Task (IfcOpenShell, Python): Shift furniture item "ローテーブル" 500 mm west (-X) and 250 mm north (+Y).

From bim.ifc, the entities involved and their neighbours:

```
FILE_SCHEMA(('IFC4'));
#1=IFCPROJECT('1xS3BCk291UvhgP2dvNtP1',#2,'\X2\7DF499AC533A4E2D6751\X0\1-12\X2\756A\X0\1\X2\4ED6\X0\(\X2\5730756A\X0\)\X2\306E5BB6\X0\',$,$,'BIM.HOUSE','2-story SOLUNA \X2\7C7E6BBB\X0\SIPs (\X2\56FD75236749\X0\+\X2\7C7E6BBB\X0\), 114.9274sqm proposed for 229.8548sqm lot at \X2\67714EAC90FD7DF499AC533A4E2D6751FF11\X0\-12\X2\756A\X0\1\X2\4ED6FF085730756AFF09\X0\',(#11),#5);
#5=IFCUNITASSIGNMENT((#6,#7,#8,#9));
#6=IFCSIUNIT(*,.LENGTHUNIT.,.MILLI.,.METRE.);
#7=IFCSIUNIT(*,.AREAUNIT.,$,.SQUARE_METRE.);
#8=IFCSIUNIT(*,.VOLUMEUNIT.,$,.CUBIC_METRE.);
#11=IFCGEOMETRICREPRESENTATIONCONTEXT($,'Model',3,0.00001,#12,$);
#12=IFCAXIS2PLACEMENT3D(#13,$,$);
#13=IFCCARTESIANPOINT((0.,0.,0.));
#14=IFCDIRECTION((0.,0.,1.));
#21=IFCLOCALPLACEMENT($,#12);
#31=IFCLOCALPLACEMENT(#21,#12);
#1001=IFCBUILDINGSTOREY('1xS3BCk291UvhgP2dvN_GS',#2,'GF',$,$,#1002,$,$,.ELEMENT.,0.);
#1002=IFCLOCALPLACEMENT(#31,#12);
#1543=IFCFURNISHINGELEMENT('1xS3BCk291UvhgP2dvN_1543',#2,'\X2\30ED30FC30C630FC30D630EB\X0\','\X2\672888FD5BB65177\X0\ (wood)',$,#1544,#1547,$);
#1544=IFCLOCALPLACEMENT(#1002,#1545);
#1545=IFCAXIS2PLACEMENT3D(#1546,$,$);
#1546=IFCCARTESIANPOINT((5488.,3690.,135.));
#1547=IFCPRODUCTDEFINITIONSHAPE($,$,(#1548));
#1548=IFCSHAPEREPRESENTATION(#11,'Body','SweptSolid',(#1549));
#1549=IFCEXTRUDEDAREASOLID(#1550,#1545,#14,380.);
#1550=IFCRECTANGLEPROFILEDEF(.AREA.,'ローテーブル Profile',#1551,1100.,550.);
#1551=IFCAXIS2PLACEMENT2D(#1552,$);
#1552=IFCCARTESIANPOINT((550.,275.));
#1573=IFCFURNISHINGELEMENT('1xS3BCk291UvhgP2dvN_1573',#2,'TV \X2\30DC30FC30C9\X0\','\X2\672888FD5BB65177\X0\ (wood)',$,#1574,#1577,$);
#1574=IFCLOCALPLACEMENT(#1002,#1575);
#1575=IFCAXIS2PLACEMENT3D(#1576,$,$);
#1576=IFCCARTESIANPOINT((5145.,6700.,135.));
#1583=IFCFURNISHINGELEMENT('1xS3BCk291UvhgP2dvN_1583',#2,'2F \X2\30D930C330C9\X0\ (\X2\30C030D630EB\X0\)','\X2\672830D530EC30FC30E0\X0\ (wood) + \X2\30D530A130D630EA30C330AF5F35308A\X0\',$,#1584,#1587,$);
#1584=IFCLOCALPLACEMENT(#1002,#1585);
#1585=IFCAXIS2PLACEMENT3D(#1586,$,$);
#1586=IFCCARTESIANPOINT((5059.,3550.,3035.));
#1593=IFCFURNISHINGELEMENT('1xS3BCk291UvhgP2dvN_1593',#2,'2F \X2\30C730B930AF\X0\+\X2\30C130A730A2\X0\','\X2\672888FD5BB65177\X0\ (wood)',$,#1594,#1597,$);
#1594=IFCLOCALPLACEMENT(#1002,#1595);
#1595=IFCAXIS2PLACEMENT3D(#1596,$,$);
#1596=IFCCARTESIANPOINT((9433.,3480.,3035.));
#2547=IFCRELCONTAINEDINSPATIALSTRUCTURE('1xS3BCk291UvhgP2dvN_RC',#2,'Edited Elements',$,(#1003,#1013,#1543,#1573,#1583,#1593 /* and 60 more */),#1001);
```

```python
import ifcopenshell
import ifcopenshell.api.geometry
import ifcopenshell.util.placement
import ifcopenshell.util.unit

model = ifcopenshell.open("bim.ifc")
unit_scale = ifcopenshell.util.unit.calculate_unit_scale(model)

item = model.by_guid("1xS3BCk291UvhgP2dvN_1543")
matrix = ifcopenshell.util.placement.get_local_placement(item.ObjectPlacement)
matrix[0, 3] -= 0.5 / unit_scale
matrix[1, 3] += 0.25 / unit_scale
ifcopenshell.api.geometry.edit_object_placement(model, product=item, matrix=matrix, is_si=False)

print(ifcopenshell.util.placement.get_local_placement(item.ObjectPlacement).round(3) + 0.0)

model.write("bim_v2.ifc")
```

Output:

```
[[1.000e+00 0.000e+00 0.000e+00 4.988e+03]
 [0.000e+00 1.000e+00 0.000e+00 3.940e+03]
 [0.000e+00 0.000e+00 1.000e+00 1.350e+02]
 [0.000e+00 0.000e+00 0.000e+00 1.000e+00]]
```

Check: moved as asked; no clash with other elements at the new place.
